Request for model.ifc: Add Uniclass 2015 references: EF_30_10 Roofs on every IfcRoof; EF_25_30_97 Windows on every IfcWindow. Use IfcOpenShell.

First a look at what the model holds.

```python
import ifcopenshell

model = ifcopenshell.open("model.ifc")
print(model.schema)
print("classifications:", [c.Name for c in model.by_type("IfcClassification")])
for ifc_class in ("IfcDoor", "IfcRoof", "IfcStair", "IfcWall", "IfcWindow"):
    print(ifc_class, len(model.by_type(ifc_class)))
```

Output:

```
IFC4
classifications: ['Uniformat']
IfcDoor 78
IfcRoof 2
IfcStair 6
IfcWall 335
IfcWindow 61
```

```python
import ifcopenshell
import ifcopenshell.api.classification

model = ifcopenshell.open("model.ifc")

system = ifcopenshell.api.classification.add_classification(model, classification="Uniclass 2015")

codes = {
    "IfcRoof": ("EF_30_10", "Roofs"),
    "IfcWindow": ("EF_25_30_97", "Windows"),
}
for ifc_class, (code, name) in codes.items():
    products = model.by_type(ifc_class)
    ifcopenshell.api.classification.add_reference(
        model, products=products, classification=system, identification=code, name=name
    )
    print(code, len(products))

model.write("model_v2.ifc")
```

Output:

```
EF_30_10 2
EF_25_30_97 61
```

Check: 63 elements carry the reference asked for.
